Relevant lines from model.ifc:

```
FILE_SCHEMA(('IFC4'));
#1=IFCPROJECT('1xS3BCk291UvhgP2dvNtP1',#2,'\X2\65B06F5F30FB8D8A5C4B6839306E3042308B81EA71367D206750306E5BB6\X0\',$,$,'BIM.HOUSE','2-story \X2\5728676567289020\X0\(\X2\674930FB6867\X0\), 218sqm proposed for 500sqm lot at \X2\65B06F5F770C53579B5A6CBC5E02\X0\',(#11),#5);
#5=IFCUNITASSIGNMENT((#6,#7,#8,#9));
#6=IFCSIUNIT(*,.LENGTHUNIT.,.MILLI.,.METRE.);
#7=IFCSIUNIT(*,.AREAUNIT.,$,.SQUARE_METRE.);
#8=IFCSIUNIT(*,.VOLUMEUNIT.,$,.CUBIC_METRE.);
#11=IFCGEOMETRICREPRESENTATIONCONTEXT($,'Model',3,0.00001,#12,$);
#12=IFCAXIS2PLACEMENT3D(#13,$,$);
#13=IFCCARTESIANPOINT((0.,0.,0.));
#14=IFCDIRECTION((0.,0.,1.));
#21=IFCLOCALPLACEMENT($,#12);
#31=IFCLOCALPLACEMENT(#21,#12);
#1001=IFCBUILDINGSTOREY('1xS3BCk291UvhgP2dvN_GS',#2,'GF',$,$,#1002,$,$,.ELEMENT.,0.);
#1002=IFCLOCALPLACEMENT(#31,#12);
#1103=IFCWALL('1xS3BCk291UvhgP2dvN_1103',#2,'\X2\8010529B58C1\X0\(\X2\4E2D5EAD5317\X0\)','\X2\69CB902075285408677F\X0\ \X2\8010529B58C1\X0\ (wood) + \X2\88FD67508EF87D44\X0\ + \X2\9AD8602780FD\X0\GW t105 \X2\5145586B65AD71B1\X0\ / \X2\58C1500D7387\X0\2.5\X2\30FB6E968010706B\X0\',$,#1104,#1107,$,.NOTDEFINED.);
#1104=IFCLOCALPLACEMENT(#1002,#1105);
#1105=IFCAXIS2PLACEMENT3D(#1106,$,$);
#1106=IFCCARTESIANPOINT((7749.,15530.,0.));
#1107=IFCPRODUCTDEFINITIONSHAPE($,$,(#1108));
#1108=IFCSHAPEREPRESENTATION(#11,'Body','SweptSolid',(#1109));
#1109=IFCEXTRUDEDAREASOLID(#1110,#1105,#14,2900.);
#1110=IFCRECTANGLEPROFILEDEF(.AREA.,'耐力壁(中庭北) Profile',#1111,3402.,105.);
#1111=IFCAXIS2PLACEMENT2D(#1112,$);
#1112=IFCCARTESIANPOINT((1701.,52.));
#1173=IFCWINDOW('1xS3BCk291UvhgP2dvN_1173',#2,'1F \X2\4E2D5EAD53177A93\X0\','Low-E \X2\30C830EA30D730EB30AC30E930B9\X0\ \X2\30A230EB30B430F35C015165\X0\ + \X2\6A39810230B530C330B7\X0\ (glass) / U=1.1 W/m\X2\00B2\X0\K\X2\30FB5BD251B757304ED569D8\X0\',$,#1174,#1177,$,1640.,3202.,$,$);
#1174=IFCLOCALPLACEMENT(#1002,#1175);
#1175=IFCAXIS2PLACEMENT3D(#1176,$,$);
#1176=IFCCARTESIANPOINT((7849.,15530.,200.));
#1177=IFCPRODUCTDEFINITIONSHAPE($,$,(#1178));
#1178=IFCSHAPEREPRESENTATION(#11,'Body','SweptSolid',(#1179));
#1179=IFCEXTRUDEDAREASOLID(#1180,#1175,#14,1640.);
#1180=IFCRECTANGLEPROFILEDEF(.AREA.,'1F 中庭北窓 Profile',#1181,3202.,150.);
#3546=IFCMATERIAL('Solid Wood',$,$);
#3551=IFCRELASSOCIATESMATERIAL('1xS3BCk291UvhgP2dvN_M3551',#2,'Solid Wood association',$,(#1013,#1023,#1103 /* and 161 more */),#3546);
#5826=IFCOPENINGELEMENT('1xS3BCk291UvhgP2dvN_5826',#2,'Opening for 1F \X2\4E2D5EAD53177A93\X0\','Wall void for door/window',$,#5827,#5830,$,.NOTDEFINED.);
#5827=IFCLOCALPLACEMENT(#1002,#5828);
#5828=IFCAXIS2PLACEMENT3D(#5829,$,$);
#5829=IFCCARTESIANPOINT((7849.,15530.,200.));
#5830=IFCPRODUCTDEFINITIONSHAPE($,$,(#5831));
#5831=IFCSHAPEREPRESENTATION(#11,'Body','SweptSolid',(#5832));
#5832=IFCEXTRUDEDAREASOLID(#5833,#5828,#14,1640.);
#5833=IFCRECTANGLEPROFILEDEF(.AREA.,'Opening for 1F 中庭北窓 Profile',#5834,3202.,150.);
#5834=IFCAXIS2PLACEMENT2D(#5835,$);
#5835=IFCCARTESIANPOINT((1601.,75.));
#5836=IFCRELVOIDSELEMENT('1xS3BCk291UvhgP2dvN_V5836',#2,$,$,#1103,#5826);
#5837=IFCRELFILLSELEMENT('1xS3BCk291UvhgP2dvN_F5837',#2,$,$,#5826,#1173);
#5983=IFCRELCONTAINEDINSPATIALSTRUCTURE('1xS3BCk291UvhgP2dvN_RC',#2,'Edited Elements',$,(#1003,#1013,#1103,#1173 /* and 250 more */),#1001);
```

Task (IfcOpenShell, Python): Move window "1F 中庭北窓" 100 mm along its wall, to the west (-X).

```python
import ifcopenshell
import ifcopenshell.api.geometry
import ifcopenshell.util.placement
import ifcopenshell.util.unit

model = ifcopenshell.open("model.ifc")
unit_scale = ifcopenshell.util.unit.calculate_unit_scale(model)

window = model.by_guid("1xS3BCk291UvhgP2dvN_1173")
opening = window.FillsVoids[0].RelatingOpeningElement
wall = opening.VoidsElements[0].RelatingBuildingElement

wall_matrix = ifcopenshell.util.placement.get_local_placement(wall.ObjectPlacement)
shift = wall_matrix[:3, 0] * -0.1 / unit_scale
before = ifcopenshell.util.placement.get_local_placement(window.ObjectPlacement)[:3, 3].copy()

# The window is not placed relative to its opening, so move both.
for product in (opening, window):
    matrix = ifcopenshell.util.placement.get_local_placement(product.ObjectPlacement)
    matrix[:3, 3] += shift
    ifcopenshell.api.geometry.edit_object_placement(model, product=product, matrix=matrix, is_si=False)

after = ifcopenshell.util.placement.get_local_placement(window.ObjectPlacement)[:3, 3]
print("window moved by", (after - before).round(3) + 0.0)

model.write("model_rev.ifc")
```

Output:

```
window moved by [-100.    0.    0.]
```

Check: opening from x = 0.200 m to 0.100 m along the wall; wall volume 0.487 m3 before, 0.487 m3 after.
